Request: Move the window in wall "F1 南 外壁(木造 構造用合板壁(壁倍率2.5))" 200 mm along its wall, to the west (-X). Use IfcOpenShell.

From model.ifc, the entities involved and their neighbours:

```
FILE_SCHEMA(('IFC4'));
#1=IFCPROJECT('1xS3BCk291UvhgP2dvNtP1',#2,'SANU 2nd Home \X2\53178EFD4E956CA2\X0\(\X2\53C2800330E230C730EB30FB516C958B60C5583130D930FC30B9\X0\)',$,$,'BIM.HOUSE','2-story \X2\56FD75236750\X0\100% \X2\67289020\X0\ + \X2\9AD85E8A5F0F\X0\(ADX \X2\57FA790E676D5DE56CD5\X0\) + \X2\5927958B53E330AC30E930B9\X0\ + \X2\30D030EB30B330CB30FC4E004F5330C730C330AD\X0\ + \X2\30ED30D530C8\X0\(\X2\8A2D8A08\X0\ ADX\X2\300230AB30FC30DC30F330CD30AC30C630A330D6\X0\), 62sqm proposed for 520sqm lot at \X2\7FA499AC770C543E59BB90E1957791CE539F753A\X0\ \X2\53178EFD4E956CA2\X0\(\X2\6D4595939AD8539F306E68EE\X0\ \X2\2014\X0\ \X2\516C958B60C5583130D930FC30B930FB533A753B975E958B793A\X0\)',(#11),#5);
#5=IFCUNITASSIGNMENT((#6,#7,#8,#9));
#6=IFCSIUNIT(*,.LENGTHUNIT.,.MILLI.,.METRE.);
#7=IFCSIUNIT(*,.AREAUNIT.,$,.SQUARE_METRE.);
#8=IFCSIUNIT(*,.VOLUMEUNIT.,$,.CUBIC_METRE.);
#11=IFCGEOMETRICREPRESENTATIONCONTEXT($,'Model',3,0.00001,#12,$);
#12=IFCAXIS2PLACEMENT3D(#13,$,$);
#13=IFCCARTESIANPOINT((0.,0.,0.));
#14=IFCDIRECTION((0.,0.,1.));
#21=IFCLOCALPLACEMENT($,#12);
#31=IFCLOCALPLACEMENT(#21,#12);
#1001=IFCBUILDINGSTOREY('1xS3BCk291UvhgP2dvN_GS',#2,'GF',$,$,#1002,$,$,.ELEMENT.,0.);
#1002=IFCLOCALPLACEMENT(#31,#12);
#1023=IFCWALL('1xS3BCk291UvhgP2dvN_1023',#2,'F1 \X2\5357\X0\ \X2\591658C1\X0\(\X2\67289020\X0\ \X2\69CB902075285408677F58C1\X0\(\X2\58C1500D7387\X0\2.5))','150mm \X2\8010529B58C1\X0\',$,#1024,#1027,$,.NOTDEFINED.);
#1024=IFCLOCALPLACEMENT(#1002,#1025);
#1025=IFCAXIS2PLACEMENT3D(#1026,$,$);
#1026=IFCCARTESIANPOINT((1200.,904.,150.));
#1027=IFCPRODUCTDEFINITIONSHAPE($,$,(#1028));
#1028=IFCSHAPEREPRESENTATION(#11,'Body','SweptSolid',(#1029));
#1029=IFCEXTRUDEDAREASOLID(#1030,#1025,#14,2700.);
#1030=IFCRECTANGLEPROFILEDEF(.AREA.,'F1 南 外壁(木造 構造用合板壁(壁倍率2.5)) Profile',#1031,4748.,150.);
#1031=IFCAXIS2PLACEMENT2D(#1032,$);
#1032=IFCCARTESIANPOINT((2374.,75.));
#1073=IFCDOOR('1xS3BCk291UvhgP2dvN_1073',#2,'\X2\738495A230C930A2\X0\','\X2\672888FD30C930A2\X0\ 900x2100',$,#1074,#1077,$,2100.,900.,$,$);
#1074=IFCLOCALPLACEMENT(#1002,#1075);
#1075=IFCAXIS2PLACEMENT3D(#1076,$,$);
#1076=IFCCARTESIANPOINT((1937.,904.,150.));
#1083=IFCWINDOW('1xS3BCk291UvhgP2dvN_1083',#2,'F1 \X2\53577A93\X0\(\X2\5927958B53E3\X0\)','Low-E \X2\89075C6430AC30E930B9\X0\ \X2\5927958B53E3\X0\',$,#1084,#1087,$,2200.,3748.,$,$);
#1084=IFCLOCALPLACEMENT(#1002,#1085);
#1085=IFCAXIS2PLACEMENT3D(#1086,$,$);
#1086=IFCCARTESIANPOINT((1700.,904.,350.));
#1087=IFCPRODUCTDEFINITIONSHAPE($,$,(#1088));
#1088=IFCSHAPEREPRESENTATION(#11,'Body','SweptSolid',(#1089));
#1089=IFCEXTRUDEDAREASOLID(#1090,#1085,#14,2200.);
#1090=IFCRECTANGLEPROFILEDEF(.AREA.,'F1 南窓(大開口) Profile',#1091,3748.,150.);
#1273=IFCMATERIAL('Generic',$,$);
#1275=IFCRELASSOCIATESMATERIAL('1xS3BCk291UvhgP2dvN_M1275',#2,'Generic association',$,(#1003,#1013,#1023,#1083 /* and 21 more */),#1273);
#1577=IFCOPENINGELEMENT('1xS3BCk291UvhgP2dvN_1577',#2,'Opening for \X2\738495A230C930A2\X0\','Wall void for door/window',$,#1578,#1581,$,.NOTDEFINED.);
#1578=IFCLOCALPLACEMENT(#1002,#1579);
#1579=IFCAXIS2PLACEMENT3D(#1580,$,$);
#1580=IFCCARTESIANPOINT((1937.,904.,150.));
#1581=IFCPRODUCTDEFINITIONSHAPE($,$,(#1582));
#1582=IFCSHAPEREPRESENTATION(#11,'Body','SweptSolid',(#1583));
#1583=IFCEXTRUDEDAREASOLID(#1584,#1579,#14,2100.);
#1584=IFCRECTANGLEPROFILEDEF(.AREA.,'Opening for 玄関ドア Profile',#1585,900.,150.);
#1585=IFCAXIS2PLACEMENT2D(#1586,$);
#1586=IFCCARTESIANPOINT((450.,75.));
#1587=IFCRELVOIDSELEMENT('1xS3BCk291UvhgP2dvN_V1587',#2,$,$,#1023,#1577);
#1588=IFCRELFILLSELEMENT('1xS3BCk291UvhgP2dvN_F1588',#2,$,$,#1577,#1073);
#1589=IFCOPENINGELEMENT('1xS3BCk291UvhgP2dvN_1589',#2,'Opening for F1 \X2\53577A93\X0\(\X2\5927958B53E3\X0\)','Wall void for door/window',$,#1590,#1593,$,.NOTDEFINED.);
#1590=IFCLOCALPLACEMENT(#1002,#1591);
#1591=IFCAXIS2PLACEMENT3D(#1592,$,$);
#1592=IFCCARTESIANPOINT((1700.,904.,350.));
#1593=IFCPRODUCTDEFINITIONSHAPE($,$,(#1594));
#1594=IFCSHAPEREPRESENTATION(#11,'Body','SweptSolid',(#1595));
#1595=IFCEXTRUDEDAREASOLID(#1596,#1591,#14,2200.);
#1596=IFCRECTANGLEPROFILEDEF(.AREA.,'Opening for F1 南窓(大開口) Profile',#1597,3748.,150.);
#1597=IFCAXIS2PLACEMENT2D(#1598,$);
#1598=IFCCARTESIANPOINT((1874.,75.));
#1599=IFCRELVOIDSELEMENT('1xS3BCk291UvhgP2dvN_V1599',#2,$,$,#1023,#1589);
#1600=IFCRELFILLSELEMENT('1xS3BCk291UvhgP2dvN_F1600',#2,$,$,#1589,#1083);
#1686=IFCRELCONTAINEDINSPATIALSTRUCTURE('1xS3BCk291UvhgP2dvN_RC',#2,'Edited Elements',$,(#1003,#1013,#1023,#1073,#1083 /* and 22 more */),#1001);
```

```python
import ifcopenshell
import ifcopenshell.api.geometry
import ifcopenshell.util.placement

model = ifcopenshell.open("model.ifc")

window = model.by_guid("1xS3BCk291UvhgP2dvN_1083")
opening = window.FillsVoids[0].RelatingOpeningElement
wall = opening.VoidsElements[0].RelatingBuildingElement

wall_matrix = ifcopenshell.util.placement.get_local_placement(wall.ObjectPlacement)
shift = wall_matrix[:3, 0] * -200.0
before = ifcopenshell.util.placement.get_local_placement(window.ObjectPlacement)[:3, 3].copy()

# The window is not placed relative to its opening, so move both.
for product in (opening, window):
    matrix = ifcopenshell.util.placement.get_local_placement(product.ObjectPlacement)
    matrix[:3, 3] += shift
    ifcopenshell.api.geometry.edit_object_placement(model, product=product, matrix=matrix, is_si=False)

after = ifcopenshell.util.placement.get_local_placement(window.ObjectPlacement)[:3, 3]
print("window moved by", (after - before).round(3) + 0.0)

model.write("model_rev.ifc")
```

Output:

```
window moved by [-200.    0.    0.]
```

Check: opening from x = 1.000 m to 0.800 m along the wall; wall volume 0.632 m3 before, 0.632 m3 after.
